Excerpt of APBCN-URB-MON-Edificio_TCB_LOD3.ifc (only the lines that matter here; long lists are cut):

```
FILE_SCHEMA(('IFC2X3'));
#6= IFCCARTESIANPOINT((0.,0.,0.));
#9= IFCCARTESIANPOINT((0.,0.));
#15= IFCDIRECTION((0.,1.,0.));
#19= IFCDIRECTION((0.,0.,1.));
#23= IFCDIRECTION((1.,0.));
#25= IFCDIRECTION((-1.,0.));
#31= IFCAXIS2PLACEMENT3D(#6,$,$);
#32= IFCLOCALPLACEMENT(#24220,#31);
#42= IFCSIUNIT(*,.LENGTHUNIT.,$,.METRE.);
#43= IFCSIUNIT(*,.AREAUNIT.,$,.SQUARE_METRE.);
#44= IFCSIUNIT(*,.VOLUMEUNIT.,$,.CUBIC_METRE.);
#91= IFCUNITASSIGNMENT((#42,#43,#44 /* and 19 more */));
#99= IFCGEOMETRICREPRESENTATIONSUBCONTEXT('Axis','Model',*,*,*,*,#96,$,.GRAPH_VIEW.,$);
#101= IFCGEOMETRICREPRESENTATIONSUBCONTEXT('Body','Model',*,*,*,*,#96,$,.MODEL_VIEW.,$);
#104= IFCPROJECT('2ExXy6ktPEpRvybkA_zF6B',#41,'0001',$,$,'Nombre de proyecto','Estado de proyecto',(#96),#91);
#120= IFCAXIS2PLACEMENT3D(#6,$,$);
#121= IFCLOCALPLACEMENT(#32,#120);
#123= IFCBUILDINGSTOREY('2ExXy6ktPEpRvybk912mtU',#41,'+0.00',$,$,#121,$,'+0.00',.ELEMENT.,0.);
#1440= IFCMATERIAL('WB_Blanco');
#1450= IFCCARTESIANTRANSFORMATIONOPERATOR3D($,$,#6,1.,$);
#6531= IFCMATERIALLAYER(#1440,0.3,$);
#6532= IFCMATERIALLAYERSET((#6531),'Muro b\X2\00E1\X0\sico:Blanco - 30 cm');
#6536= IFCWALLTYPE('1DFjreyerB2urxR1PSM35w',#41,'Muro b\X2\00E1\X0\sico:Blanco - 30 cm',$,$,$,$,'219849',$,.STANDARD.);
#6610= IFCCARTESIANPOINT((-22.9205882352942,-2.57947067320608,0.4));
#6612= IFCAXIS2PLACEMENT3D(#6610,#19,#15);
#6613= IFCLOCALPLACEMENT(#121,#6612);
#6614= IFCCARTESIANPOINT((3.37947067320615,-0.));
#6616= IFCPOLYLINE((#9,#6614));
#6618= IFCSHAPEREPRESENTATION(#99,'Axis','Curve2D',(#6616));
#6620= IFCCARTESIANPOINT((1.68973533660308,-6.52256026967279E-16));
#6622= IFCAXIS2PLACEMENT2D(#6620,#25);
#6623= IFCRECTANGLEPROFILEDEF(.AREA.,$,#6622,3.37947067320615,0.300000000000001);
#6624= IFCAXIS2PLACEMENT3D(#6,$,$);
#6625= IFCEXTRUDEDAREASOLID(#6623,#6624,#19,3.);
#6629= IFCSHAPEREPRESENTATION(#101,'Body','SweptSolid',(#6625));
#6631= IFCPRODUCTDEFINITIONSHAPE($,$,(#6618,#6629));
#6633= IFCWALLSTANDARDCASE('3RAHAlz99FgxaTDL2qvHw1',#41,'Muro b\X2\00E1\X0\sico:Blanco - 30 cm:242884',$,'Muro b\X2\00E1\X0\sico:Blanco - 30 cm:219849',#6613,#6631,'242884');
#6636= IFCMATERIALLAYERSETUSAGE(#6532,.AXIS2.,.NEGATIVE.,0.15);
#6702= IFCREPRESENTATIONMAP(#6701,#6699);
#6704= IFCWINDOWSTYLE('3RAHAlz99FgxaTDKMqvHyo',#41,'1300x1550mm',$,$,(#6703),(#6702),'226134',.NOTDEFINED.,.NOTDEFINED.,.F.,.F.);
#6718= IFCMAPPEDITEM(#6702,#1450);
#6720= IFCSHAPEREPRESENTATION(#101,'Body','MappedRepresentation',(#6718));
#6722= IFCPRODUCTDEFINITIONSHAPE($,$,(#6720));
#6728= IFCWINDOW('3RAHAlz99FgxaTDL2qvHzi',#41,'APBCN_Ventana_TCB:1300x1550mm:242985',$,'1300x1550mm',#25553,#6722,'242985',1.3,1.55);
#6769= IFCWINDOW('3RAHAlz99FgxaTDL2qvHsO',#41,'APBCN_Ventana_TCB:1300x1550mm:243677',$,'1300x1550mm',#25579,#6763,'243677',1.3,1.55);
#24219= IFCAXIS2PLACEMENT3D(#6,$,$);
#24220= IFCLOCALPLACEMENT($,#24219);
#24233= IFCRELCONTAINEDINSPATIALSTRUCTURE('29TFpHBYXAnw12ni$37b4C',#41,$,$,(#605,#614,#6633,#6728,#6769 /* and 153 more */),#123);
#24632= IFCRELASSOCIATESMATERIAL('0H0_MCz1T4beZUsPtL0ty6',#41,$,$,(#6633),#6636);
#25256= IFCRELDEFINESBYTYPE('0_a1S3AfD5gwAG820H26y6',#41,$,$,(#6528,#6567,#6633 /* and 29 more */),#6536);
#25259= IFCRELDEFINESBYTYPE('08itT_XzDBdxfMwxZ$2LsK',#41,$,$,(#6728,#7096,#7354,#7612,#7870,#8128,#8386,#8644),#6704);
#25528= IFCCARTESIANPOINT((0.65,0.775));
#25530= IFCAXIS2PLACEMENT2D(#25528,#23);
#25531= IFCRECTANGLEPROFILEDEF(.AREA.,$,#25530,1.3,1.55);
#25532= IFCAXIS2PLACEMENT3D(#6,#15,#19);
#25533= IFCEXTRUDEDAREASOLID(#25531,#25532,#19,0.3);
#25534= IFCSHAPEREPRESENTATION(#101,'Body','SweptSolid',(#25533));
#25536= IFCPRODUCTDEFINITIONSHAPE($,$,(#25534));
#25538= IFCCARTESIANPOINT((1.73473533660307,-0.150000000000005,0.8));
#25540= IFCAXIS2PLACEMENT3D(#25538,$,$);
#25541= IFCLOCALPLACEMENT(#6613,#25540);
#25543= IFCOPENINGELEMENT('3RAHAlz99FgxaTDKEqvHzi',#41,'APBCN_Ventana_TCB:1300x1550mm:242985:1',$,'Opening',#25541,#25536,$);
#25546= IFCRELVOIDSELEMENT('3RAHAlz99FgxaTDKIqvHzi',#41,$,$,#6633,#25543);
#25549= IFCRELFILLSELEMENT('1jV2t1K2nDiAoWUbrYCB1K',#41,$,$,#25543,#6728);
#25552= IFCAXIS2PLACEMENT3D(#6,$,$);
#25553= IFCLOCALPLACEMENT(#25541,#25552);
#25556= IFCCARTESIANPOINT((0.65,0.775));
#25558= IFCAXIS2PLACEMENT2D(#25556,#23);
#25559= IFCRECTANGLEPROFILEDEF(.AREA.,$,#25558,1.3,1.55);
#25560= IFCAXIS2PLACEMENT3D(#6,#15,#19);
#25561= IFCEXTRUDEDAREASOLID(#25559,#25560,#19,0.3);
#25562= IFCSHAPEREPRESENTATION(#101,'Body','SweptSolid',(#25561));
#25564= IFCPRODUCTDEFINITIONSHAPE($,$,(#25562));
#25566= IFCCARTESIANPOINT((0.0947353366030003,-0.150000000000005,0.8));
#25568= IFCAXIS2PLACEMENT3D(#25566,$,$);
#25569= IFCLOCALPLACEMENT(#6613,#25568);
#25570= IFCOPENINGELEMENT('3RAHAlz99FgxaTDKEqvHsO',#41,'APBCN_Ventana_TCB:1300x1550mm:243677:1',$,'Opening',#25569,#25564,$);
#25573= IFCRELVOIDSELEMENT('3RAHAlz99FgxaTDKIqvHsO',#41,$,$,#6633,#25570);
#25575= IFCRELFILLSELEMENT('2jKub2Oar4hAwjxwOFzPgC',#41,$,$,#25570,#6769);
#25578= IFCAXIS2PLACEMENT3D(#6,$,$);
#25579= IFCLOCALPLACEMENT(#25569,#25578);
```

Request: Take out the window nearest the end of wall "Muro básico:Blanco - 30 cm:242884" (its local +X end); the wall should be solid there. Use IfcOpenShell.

```python
import ifcopenshell
import ifcopenshell.api.feature
import ifcopenshell.api.root
import ifcopenshell.geom
import ifcopenshell.util.shape

model = ifcopenshell.open("APBCN-URB-MON-Edificio_TCB_LOD3.ifc")
settings = ifcopenshell.geom.settings()


def volume(element):
    """Net volume in cubic metres, openings subtracted."""
    shape = ifcopenshell.geom.create_shape(settings, element)
    return ifcopenshell.util.shape.get_volume(shape.geometry)


window = model.by_guid("3RAHAlz99FgxaTDL2qvHzi")
opening = window.FillsVoids[0].RelatingOpeningElement
wall = opening.VoidsElements[0].RelatingBuildingElement
before = volume(wall)

ifcopenshell.api.root.remove_product(model, product=window)
ifcopenshell.api.feature.remove_feature(model, feature=opening)

after = volume(wall)

print(f"wall volume {before:.3f} -> {after:.3f} m3")

model.write("APBCN-URB-MON-Edificio_TCB_LOD3_edited.ifc")
```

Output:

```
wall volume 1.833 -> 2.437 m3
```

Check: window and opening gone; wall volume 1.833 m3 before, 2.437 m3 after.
